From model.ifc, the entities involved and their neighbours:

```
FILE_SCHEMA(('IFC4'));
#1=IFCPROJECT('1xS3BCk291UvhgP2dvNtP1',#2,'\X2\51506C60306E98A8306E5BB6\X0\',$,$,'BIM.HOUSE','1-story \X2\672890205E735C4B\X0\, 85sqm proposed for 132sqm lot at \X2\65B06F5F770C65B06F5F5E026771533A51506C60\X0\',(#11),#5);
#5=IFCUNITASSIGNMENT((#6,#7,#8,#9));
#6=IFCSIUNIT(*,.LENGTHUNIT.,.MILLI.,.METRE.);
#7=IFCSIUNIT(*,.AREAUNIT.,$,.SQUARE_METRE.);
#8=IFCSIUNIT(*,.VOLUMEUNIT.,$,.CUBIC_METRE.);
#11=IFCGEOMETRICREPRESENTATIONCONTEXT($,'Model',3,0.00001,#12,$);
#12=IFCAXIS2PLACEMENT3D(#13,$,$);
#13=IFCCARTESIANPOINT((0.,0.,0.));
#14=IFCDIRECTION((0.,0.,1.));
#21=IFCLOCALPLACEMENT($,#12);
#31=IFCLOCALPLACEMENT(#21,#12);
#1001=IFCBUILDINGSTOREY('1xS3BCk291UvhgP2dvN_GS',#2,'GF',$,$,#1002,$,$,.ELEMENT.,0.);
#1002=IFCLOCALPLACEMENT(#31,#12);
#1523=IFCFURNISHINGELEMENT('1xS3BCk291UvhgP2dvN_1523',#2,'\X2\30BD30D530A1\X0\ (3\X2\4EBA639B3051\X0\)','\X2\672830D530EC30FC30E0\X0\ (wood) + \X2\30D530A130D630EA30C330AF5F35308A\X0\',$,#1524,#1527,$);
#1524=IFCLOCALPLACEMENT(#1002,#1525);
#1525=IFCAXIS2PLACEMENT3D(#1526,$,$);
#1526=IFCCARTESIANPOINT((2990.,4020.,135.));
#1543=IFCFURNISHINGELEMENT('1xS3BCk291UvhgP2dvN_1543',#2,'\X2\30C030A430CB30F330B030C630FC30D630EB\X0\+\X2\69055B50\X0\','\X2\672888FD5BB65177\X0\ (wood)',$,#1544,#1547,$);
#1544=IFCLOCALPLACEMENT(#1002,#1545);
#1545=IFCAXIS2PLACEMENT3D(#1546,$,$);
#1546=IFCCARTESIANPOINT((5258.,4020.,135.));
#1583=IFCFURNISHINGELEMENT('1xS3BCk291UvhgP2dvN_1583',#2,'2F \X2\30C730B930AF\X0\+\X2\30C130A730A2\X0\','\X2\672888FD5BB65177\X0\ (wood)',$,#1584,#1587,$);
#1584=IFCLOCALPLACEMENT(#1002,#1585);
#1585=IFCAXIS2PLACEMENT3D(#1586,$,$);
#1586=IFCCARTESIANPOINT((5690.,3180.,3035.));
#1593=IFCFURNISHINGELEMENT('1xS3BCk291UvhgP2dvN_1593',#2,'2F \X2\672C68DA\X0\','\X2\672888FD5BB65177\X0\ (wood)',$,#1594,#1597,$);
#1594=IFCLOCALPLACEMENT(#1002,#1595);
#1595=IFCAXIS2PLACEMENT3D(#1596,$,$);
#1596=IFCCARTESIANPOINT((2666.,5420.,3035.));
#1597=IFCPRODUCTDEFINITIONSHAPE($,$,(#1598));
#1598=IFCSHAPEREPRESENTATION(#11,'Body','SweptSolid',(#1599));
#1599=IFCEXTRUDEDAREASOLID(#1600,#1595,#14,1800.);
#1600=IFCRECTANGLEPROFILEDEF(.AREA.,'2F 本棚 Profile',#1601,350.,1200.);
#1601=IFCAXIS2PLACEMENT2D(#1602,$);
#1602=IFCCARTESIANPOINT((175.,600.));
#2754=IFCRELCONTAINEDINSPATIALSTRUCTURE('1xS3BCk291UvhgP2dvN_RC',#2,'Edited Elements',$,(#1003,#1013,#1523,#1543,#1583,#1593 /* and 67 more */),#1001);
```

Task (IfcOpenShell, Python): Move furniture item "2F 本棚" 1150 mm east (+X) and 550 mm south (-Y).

```python
import ifcopenshell
import ifcopenshell.api.geometry
import ifcopenshell.util.placement

model = ifcopenshell.open("model.ifc")

item = model.by_guid("1xS3BCk291UvhgP2dvN_1593")
matrix = ifcopenshell.util.placement.get_local_placement(item.ObjectPlacement)
matrix[0, 3] += 1150.0
matrix[1, 3] -= 550.0
ifcopenshell.api.geometry.edit_object_placement(model, product=item, matrix=matrix, is_si=False)

print(ifcopenshell.util.placement.get_local_placement(item.ObjectPlacement).round(3) + 0.0)

model.write("model_updated.ifc")
```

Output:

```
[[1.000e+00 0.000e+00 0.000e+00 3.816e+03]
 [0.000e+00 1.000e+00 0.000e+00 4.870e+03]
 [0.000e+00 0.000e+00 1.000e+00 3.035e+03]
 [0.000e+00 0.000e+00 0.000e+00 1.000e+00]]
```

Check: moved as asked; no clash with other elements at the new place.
